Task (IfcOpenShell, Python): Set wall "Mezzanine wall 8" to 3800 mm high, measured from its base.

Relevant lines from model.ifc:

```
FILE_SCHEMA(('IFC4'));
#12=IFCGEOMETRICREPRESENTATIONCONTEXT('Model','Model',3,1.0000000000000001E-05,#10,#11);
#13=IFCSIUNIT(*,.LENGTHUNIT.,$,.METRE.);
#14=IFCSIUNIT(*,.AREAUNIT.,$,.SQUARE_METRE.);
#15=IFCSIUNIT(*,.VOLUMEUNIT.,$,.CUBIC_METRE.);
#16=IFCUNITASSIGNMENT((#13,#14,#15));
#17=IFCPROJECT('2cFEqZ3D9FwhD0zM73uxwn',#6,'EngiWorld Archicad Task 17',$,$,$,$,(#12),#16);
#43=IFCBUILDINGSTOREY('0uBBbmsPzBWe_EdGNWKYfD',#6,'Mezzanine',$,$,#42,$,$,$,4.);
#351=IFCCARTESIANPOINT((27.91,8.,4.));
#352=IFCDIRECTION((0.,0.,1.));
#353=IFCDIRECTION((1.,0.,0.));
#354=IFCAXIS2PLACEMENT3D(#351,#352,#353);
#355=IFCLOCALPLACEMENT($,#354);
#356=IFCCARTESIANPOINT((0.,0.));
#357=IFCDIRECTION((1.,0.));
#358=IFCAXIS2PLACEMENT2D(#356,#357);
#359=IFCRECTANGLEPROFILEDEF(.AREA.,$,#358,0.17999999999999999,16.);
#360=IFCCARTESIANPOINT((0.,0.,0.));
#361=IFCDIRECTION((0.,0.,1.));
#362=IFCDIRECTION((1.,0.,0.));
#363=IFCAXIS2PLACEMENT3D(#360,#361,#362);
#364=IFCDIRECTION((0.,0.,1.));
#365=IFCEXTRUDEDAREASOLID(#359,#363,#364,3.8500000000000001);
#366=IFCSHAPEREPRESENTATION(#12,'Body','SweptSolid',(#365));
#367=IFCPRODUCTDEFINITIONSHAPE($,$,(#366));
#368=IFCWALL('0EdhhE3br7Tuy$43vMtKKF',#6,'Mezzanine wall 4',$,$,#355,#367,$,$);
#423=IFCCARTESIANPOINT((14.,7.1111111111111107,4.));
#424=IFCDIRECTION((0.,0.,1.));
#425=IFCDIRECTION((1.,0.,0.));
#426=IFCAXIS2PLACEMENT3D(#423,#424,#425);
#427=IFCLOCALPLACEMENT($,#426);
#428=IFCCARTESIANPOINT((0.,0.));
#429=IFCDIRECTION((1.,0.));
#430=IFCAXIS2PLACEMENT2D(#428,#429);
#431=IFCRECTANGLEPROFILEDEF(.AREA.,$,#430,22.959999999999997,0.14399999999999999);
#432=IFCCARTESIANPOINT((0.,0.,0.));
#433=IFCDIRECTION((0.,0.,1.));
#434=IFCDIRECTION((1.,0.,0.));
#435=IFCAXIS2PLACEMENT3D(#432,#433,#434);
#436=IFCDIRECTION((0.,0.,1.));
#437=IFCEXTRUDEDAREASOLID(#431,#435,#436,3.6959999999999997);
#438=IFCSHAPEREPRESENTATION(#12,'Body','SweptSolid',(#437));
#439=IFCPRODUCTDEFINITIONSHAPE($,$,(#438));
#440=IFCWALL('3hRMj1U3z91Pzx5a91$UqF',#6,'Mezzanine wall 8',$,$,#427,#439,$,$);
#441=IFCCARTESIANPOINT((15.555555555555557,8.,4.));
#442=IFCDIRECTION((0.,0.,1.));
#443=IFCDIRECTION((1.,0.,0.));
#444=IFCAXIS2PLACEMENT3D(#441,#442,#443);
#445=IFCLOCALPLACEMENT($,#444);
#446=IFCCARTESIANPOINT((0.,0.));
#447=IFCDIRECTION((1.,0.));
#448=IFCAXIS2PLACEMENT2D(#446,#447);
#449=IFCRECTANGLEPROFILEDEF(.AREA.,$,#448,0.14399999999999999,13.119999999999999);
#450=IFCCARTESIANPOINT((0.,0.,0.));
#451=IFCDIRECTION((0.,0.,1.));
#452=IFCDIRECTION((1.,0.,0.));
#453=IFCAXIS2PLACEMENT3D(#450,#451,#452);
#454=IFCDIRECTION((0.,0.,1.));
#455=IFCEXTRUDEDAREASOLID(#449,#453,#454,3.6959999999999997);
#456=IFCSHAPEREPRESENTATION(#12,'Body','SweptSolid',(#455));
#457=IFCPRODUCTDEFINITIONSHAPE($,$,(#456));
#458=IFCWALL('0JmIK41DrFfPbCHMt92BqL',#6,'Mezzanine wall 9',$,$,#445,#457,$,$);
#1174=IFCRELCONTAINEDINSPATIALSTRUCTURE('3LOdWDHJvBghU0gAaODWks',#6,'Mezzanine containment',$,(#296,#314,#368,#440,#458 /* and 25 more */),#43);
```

```python
import ifcopenshell
import ifcopenshell.geom
import ifcopenshell.util.shape
import ifcopenshell.util.unit

model = ifcopenshell.open("model.ifc")
unit_scale = ifcopenshell.util.unit.calculate_unit_scale(model)
settings = ifcopenshell.geom.settings()


def volume(element):
    """Net volume in cubic metres, openings subtracted."""
    shape = ifcopenshell.geom.create_shape(settings, element)
    return ifcopenshell.util.shape.get_volume(shape.geometry)


wall = model.by_guid("3hRMj1U3z91Pzx5a91$UqF")
before = volume(wall)

body = next(r for r in wall.Representation.Representations if r.RepresentationIdentifier == "Body")
solid = body.Items[0]
old_height = solid.Depth
solid.Depth = 3.8 / unit_scale
after = volume(wall)

print(f"height {old_height:g} -> {solid.Depth:g}, volume {before:.3f} -> {after:.3f} m3")

model.write("model_v2.ifc")
```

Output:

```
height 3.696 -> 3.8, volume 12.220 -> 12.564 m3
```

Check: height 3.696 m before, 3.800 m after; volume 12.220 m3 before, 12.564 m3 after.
